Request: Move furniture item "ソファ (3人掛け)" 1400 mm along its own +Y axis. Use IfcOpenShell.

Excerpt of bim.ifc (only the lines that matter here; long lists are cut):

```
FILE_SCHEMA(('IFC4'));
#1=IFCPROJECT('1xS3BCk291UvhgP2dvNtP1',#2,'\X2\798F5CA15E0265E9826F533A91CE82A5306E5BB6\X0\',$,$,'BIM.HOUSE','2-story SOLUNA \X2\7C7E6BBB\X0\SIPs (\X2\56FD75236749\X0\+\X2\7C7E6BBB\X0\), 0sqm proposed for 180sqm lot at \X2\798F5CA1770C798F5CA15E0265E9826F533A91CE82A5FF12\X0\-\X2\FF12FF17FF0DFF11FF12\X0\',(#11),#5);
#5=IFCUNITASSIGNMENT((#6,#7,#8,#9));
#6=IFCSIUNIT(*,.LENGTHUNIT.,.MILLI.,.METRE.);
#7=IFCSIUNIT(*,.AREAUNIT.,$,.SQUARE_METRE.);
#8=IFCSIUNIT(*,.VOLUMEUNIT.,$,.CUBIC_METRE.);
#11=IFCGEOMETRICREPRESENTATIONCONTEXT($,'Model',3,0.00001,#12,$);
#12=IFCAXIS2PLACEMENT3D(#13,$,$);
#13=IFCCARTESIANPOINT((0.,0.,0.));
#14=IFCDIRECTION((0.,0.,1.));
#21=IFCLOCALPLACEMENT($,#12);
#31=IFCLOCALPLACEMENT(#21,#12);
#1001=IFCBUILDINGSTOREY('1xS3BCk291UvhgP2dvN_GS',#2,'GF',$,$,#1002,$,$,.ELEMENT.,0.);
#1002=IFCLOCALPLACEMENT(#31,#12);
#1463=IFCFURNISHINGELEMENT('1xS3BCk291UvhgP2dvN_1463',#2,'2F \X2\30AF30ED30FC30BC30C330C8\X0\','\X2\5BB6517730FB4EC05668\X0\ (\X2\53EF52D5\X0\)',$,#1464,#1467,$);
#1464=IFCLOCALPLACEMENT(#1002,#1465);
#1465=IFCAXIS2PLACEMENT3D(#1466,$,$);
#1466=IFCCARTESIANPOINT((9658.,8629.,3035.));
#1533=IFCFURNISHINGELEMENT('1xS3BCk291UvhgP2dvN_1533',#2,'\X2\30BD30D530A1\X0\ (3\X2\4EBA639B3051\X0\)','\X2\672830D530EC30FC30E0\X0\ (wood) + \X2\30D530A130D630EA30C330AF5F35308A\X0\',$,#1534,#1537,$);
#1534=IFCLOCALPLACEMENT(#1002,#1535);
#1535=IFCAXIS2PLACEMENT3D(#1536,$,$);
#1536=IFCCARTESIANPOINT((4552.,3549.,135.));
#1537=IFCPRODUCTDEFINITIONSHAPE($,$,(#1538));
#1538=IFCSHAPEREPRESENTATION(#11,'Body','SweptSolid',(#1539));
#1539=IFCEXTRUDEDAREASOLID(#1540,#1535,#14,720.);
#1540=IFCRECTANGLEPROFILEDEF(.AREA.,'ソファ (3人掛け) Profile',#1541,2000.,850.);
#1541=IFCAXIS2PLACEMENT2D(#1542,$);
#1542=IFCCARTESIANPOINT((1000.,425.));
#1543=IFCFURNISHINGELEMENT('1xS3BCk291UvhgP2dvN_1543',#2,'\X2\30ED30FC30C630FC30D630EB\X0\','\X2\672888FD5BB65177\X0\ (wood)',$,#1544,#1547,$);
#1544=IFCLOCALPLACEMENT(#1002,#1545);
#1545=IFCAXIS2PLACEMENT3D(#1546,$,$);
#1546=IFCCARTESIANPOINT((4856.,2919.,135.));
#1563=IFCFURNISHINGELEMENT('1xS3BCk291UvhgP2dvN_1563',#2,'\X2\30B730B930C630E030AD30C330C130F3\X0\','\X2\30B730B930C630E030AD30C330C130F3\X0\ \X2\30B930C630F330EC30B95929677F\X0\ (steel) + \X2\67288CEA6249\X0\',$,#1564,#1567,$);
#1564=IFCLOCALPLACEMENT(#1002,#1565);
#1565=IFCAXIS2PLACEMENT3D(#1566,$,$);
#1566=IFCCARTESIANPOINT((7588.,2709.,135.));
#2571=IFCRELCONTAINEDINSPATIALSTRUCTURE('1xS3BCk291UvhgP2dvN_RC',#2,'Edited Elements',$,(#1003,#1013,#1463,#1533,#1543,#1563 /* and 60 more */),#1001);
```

```python
import ifcopenshell
import ifcopenshell.api.geometry
import ifcopenshell.util.placement
import ifcopenshell.util.unit

model = ifcopenshell.open("bim.ifc")
unit_scale = ifcopenshell.util.unit.calculate_unit_scale(model)

item = model.by_guid("1xS3BCk291UvhgP2dvN_1533")
matrix = ifcopenshell.util.placement.get_local_placement(item.ObjectPlacement)
matrix[:3, 3] += matrix[:3, 1] * 1.4 / unit_scale
ifcopenshell.api.geometry.edit_object_placement(model, product=item, matrix=matrix, is_si=False)

print(ifcopenshell.util.placement.get_local_placement(item.ObjectPlacement).round(3) + 0.0)

model.write("bim_v2.ifc")
```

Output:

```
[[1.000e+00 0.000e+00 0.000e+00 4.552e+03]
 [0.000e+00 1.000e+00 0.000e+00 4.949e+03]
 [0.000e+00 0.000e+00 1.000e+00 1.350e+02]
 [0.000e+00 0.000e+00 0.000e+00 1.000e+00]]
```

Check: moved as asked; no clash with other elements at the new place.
